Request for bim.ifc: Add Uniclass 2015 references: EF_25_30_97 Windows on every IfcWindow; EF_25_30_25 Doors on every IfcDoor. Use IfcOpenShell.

First a look at what the model holds.

```python
import ifcopenshell

model = ifcopenshell.open("bim.ifc")
print(model.schema)
print("classifications:", [c.Name for c in model.by_type("IfcClassification")])
for ifc_class in ("IfcDoor", "IfcRoof", "IfcStair", "IfcWall", "IfcWindow"):
    print(ifc_class, len(model.by_type(ifc_class)))
```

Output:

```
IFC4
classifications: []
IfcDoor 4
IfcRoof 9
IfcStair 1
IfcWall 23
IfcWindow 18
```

```python
import ifcopenshell
import ifcopenshell.api.classification

model = ifcopenshell.open("bim.ifc")

system = ifcopenshell.api.classification.add_classification(model, classification="Uniclass 2015")

codes = {
    "IfcWindow": ("EF_25_30_97", "Windows"),
    "IfcDoor": ("EF_25_30_25", "Doors"),
}
for ifc_class, (code, name) in codes.items():
    products = model.by_type(ifc_class)
    ifcopenshell.api.classification.add_reference(
        model, products=products, classification=system, identification=code, name=name
    )
    print(code, len(products))

model.write("bim-out.ifc")
```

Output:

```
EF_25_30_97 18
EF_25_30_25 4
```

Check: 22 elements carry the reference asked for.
